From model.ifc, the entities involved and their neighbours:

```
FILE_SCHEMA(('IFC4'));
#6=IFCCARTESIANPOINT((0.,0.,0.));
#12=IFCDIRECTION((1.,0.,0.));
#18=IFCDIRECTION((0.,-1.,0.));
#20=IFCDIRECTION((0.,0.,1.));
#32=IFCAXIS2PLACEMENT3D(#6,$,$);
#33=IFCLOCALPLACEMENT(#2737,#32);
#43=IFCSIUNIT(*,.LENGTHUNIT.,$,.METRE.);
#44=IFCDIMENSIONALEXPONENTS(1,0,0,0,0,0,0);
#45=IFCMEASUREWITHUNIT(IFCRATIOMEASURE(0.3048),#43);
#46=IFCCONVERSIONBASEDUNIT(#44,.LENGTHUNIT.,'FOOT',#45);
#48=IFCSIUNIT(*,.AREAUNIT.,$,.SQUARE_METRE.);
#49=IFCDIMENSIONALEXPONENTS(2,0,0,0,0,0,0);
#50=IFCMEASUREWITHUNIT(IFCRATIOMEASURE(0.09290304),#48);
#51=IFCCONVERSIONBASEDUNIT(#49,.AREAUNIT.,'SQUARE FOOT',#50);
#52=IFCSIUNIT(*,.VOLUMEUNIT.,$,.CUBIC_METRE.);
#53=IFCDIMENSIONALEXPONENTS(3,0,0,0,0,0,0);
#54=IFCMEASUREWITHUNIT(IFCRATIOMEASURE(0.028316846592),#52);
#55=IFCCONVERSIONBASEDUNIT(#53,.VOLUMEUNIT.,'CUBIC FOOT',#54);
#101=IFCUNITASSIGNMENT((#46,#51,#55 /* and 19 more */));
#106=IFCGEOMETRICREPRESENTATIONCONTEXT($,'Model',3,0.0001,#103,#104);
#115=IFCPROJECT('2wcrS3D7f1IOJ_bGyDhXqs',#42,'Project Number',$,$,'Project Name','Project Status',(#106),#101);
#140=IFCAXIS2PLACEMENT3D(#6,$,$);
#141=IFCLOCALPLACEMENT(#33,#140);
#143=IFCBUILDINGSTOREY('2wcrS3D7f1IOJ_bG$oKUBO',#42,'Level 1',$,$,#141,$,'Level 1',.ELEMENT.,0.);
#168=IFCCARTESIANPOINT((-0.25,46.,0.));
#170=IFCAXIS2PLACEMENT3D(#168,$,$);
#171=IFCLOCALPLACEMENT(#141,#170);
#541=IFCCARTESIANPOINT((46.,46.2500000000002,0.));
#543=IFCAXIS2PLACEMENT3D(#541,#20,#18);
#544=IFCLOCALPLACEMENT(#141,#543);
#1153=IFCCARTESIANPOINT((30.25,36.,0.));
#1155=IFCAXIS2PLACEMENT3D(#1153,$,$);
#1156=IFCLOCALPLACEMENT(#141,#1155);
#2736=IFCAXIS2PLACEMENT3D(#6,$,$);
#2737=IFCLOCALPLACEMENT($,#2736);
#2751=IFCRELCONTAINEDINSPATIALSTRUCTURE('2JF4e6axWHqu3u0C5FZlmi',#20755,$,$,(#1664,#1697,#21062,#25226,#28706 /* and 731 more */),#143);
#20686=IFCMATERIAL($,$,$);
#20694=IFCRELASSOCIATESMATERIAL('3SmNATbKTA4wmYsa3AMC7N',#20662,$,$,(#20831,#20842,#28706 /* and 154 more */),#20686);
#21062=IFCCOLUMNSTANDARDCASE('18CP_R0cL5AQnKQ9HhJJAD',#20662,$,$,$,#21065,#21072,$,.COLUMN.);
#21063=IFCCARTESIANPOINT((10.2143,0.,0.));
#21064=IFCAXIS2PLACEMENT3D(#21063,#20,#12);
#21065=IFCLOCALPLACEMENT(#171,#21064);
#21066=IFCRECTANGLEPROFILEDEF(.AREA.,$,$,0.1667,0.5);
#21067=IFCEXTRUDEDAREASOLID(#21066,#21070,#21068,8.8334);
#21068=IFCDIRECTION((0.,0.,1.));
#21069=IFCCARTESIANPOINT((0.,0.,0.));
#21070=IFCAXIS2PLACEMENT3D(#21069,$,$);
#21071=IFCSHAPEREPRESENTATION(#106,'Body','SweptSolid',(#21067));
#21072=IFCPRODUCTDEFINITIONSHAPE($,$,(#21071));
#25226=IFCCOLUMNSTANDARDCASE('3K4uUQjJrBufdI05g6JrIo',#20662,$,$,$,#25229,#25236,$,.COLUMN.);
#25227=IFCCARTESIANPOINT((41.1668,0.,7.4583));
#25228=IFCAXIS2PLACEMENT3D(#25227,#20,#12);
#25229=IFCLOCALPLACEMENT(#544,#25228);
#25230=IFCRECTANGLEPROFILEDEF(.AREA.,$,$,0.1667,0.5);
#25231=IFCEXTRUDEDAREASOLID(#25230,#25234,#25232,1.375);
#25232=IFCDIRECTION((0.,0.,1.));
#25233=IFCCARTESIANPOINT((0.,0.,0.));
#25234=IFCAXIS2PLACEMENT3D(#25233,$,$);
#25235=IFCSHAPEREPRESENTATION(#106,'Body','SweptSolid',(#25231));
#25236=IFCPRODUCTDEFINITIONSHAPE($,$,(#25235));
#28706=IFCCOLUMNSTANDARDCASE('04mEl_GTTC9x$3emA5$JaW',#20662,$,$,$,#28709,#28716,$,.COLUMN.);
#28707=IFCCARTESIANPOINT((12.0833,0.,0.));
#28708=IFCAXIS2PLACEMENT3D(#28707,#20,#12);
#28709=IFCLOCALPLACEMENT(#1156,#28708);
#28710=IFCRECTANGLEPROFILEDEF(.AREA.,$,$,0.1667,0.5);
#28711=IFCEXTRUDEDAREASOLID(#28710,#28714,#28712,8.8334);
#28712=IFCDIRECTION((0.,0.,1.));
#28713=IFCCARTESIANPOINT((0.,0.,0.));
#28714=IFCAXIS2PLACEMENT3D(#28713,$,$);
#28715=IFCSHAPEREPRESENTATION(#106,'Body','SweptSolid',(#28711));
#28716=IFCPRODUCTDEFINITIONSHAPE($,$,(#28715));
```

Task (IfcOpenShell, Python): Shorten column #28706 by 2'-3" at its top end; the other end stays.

```python
import ifcopenshell
import ifcopenshell.util.unit

model = ifcopenshell.open("model.ifc")
unit_scale = ifcopenshell.util.unit.calculate_unit_scale(model)

member = model.by_guid("04mEl_GTTC9x$3emA5$JaW")
change = -27 * 0.0254 / unit_scale

# The extrusion runs towards the end named, so only its depth changes.
body = next(r for r in member.Representation.Representations if r.RepresentationIdentifier == "Body")
solid = body.Items[0]
old_length = solid.Depth
solid.Depth += change

print(f"length {old_length:g} -> {solid.Depth:g}")

model.write("model_v2.ifc")
```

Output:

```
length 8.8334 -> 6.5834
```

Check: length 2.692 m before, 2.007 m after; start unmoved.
